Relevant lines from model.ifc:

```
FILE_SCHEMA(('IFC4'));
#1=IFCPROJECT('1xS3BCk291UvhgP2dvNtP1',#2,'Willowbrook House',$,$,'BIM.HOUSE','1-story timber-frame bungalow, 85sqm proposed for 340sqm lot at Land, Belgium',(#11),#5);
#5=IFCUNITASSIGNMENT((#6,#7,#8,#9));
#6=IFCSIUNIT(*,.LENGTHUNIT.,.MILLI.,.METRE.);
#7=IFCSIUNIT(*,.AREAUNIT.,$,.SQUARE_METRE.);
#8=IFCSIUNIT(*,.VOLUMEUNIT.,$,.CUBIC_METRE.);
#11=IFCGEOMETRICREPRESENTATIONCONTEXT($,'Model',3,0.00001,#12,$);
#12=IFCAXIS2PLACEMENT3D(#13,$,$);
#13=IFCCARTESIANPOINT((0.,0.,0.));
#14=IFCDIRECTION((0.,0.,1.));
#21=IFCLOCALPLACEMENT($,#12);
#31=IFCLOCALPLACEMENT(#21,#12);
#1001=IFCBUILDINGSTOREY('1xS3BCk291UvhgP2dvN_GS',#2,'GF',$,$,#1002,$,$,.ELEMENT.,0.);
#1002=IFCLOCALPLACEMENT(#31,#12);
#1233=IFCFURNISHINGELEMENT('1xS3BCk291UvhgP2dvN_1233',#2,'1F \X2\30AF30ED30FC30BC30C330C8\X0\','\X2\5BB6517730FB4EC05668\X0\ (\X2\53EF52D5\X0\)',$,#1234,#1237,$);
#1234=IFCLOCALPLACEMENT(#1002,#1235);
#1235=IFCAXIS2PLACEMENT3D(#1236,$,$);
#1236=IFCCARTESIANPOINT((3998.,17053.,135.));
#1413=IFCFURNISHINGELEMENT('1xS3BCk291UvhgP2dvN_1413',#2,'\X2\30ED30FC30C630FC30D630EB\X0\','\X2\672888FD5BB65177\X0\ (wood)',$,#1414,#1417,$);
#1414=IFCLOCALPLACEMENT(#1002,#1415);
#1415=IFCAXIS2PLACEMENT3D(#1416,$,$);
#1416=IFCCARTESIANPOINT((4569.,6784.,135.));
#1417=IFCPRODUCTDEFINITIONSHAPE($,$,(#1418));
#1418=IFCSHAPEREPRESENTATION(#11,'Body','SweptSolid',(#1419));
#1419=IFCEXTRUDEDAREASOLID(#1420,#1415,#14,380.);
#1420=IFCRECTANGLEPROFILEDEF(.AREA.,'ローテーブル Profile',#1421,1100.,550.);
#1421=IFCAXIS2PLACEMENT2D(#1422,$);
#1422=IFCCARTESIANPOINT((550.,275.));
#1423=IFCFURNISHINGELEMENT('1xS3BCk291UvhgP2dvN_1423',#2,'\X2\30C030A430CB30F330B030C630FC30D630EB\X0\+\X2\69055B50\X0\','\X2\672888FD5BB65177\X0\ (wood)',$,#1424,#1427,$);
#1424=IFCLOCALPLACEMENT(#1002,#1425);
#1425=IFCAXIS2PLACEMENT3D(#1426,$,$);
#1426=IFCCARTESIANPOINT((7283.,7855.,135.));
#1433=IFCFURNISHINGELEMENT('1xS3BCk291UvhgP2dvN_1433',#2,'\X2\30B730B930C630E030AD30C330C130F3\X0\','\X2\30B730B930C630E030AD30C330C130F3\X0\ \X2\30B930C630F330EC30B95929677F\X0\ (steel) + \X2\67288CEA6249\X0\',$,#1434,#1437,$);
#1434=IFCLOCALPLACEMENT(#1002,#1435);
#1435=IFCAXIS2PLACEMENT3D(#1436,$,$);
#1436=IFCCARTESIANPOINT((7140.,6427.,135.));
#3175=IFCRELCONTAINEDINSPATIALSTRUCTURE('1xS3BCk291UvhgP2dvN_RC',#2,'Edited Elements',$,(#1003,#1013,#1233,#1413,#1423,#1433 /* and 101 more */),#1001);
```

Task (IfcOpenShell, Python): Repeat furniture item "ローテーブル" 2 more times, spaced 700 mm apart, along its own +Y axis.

```python
import ifcopenshell
import ifcopenshell.api.geometry
import ifcopenshell.api.root
import ifcopenshell.util.element
import ifcopenshell.util.placement
import ifcopenshell.util.unit

model = ifcopenshell.open("model.ifc")
unit_scale = ifcopenshell.util.unit.calculate_unit_scale(model)


def reuse_history(source, copy):
    """copy_class also copies each property set's owner history, people and application; keep the originals."""
    for rel in copy.IsDefinedBy:
        if rel.is_a("IfcRelDefinesByProperties") and (history := rel.RelatingPropertyDefinition.OwnerHistory):
            rel.RelatingPropertyDefinition.OwnerHistory = source.OwnerHistory
            ifcopenshell.util.element.remove_deep2(model, history)


source = model.by_guid("1xS3BCk291UvhgP2dvN_1413")
base = ifcopenshell.util.placement.get_local_placement(source.ObjectPlacement)
step = base[:3, 1] * 0.7 / unit_scale

for i in range(1, 3):
    copy = ifcopenshell.api.root.copy_class(model, product=source)
    copy.Representation = ifcopenshell.util.element.copy_deep(
        model, source.Representation, exclude=["IfcGeometricRepresentationContext", "IfcRepresentationMap"]
    )
    reuse_history(source, copy)
    matrix = base.copy()
    matrix[:3, 3] += i * step
    print("added at", matrix[:3, 3].round(3) + 0.0)
    ifcopenshell.api.geometry.edit_object_placement(model, product=copy, matrix=matrix, is_si=False)

model.write("model-out.ifc")
```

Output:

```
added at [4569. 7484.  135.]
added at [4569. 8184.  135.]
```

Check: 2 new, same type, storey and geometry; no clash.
